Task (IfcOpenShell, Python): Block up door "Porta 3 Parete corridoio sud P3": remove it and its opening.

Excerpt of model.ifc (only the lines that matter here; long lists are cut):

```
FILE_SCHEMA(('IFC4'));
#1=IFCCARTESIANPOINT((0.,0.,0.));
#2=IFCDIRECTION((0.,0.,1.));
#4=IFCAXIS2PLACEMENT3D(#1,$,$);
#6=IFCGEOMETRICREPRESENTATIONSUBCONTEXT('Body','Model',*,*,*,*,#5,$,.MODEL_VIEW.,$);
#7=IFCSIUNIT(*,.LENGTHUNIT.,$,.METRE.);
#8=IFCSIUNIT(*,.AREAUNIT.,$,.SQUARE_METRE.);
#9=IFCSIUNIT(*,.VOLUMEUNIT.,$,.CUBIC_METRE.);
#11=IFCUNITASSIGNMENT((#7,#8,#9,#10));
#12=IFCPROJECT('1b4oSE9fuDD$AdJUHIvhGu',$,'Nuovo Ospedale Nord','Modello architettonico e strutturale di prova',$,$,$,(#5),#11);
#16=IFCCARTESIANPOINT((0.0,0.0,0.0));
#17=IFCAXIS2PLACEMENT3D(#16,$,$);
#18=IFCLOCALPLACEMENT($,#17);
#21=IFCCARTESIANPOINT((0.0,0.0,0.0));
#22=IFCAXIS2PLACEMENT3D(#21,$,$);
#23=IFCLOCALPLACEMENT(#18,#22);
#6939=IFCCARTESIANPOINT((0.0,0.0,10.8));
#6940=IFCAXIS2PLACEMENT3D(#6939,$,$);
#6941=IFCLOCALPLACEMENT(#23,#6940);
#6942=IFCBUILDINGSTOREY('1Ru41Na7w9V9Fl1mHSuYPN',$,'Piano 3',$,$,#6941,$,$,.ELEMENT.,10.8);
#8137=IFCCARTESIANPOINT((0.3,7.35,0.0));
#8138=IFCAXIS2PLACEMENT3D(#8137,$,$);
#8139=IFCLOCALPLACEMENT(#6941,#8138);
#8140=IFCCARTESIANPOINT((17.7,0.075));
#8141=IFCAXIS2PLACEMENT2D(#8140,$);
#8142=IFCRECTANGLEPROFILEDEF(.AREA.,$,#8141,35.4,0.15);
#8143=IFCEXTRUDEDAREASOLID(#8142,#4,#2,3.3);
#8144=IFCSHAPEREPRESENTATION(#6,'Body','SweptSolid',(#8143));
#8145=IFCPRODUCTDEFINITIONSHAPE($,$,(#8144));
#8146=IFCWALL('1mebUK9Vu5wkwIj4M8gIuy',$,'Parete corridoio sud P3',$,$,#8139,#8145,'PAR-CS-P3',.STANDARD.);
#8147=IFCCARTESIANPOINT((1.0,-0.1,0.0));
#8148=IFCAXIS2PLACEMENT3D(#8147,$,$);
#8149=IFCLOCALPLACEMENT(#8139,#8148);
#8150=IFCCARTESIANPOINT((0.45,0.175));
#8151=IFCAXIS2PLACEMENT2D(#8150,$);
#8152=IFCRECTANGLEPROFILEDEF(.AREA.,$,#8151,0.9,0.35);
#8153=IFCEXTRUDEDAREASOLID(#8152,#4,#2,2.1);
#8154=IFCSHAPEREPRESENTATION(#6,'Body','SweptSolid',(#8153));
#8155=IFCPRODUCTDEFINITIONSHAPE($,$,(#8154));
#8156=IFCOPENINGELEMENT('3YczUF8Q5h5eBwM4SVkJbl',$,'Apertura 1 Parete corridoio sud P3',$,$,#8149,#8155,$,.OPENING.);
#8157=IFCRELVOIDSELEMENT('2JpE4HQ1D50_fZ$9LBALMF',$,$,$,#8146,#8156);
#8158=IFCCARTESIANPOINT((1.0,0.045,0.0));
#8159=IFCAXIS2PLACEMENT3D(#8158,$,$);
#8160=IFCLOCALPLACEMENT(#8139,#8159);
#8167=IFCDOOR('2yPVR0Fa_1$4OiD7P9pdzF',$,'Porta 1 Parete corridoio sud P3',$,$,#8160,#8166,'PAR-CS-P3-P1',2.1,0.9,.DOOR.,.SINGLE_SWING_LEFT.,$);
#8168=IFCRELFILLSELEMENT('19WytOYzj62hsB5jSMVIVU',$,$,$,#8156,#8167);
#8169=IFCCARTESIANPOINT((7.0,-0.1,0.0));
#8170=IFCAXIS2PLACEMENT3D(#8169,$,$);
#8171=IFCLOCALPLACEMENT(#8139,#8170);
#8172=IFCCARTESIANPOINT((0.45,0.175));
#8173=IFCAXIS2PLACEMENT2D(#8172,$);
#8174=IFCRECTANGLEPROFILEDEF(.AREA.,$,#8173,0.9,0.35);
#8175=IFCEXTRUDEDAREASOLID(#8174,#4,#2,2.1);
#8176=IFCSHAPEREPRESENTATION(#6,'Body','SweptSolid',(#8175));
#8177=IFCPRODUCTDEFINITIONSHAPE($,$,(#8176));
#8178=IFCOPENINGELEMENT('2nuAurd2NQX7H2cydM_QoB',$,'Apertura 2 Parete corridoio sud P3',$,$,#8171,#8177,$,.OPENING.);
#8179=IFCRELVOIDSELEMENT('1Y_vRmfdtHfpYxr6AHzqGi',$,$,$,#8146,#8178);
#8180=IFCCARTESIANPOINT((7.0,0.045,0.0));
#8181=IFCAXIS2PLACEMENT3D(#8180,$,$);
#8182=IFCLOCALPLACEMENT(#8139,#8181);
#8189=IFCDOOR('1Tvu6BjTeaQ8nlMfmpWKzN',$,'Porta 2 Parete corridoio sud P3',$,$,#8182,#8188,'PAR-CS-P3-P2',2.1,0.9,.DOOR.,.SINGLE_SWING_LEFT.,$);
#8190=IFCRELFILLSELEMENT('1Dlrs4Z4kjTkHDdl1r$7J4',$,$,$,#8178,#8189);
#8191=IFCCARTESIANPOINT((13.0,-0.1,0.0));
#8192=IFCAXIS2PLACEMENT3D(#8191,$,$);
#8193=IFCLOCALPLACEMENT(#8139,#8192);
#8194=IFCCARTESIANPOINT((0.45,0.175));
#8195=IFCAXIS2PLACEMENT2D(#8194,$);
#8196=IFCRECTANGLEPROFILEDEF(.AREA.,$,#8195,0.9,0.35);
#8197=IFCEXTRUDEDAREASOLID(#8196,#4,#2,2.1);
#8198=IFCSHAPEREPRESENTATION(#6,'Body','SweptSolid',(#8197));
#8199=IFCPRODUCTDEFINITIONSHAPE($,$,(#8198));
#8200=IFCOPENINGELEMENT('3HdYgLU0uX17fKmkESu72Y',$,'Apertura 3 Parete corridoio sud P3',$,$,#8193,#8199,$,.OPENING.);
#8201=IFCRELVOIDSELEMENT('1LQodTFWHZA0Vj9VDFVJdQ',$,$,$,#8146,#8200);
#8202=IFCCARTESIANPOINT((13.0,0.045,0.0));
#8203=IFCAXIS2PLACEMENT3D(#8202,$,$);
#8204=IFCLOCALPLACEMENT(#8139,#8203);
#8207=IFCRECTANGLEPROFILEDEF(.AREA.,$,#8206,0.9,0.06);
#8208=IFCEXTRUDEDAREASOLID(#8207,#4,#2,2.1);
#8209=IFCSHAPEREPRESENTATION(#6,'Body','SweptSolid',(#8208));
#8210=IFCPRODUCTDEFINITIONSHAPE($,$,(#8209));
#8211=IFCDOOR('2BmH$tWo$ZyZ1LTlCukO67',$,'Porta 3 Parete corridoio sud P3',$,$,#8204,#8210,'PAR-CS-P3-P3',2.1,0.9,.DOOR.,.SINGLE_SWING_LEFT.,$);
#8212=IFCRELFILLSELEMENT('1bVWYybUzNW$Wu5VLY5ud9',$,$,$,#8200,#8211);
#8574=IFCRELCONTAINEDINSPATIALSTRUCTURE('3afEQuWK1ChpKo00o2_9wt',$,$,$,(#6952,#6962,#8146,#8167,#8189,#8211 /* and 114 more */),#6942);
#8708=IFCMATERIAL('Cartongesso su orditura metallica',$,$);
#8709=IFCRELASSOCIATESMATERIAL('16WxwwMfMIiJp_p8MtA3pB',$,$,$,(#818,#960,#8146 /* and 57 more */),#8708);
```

```python
import ifcopenshell
import ifcopenshell.api.feature
import ifcopenshell.api.root
import ifcopenshell.geom
import ifcopenshell.util.shape

model = ifcopenshell.open("model.ifc")
settings = ifcopenshell.geom.settings()


def volume(element):
    """Net volume in cubic metres, openings subtracted."""
    shape = ifcopenshell.geom.create_shape(settings, element)
    return ifcopenshell.util.shape.get_volume(shape.geometry)


door = model.by_guid("2BmH$tWo$ZyZ1LTlCukO67")
opening = door.FillsVoids[0].RelatingOpeningElement
wall = opening.VoidsElements[0].RelatingBuildingElement
before = volume(wall)

ifcopenshell.api.root.remove_product(model, product=door)
ifcopenshell.api.feature.remove_feature(model, feature=opening)

after = volume(wall)

print(f"wall volume {before:.3f} -> {after:.3f} m3")

model.write("model-out.ifc")
```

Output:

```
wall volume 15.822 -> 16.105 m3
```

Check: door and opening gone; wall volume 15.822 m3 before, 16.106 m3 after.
